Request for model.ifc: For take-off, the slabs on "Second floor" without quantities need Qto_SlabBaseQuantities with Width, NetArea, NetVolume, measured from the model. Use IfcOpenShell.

First a look at what the model holds.

```python
import ifcopenshell
import ifcopenshell.util.element
import ifcopenshell.util.unit

model = ifcopenshell.open("model.ifc")
print(model.schema)
for unit_type in ("LENGTHUNIT", "AREAUNIT", "VOLUMEUNIT"):
    print(unit_type, ifcopenshell.util.unit.calculate_unit_scale(model, unit_type))
storey = next(s for s in model.by_type("IfcBuildingStorey") if s.Name == "Second floor")
slabs = [e for e in ifcopenshell.util.element.get_decomposition(storey) if e.is_a("IfcSlab")]
for e in sorted(slabs, key=lambda e: e.id()):
    print(e.id(), e.is_a(), e.Name, list(ifcopenshell.util.element.get_psets(e, qtos_only=True)), sep=" | ")
```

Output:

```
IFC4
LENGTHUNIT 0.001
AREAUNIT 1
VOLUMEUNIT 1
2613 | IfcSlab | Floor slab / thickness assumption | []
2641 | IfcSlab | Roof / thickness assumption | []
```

```python
import ifcopenshell
import ifcopenshell.api.pset
import ifcopenshell.geom
import ifcopenshell.util.element
import ifcopenshell.util.shape
import ifcopenshell.util.unit

model = ifcopenshell.open("model.ifc")
unit_scale = ifcopenshell.util.unit.calculate_unit_scale(model)
area_scale = ifcopenshell.util.unit.calculate_unit_scale(model, "AREAUNIT")
volume_scale = ifcopenshell.util.unit.calculate_unit_scale(model, "VOLUMEUNIT")
settings = ifcopenshell.geom.settings()

storey = next(s for s in model.by_type("IfcBuildingStorey") if s.Name == "Second floor")
slabs = [e for e in ifcopenshell.util.element.get_decomposition(storey) if e.is_a("IfcSlab")]

for e in sorted(slabs, key=lambda e: e.id()):
    if ifcopenshell.util.element.get_psets(e, qtos_only=True, should_inherit=False):
        continue
    # Geometry comes back in metres, in the element's own axes.
    shape = ifcopenshell.geom.create_shape(settings, e)
    values = {
        "Width": ifcopenshell.util.shape.get_z(shape.geometry) / unit_scale,
        "NetArea": ifcopenshell.util.shape.get_footprint_area(shape.geometry) / area_scale,
        "NetVolume": ifcopenshell.util.shape.get_volume(shape.geometry) / volume_scale,
    }
    qto = ifcopenshell.api.pset.add_qto(model, product=e, name="Qto_SlabBaseQuantities")
    ifcopenshell.api.pset.edit_qto(model, qto=qto, properties=values)
    print(e.id(), {k: round(v, 3) for k, v in values.items()})

model.write("model_edited.ifc")
```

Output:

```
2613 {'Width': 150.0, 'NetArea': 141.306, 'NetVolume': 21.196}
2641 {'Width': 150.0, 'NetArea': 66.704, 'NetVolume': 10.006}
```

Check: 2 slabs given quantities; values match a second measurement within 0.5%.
